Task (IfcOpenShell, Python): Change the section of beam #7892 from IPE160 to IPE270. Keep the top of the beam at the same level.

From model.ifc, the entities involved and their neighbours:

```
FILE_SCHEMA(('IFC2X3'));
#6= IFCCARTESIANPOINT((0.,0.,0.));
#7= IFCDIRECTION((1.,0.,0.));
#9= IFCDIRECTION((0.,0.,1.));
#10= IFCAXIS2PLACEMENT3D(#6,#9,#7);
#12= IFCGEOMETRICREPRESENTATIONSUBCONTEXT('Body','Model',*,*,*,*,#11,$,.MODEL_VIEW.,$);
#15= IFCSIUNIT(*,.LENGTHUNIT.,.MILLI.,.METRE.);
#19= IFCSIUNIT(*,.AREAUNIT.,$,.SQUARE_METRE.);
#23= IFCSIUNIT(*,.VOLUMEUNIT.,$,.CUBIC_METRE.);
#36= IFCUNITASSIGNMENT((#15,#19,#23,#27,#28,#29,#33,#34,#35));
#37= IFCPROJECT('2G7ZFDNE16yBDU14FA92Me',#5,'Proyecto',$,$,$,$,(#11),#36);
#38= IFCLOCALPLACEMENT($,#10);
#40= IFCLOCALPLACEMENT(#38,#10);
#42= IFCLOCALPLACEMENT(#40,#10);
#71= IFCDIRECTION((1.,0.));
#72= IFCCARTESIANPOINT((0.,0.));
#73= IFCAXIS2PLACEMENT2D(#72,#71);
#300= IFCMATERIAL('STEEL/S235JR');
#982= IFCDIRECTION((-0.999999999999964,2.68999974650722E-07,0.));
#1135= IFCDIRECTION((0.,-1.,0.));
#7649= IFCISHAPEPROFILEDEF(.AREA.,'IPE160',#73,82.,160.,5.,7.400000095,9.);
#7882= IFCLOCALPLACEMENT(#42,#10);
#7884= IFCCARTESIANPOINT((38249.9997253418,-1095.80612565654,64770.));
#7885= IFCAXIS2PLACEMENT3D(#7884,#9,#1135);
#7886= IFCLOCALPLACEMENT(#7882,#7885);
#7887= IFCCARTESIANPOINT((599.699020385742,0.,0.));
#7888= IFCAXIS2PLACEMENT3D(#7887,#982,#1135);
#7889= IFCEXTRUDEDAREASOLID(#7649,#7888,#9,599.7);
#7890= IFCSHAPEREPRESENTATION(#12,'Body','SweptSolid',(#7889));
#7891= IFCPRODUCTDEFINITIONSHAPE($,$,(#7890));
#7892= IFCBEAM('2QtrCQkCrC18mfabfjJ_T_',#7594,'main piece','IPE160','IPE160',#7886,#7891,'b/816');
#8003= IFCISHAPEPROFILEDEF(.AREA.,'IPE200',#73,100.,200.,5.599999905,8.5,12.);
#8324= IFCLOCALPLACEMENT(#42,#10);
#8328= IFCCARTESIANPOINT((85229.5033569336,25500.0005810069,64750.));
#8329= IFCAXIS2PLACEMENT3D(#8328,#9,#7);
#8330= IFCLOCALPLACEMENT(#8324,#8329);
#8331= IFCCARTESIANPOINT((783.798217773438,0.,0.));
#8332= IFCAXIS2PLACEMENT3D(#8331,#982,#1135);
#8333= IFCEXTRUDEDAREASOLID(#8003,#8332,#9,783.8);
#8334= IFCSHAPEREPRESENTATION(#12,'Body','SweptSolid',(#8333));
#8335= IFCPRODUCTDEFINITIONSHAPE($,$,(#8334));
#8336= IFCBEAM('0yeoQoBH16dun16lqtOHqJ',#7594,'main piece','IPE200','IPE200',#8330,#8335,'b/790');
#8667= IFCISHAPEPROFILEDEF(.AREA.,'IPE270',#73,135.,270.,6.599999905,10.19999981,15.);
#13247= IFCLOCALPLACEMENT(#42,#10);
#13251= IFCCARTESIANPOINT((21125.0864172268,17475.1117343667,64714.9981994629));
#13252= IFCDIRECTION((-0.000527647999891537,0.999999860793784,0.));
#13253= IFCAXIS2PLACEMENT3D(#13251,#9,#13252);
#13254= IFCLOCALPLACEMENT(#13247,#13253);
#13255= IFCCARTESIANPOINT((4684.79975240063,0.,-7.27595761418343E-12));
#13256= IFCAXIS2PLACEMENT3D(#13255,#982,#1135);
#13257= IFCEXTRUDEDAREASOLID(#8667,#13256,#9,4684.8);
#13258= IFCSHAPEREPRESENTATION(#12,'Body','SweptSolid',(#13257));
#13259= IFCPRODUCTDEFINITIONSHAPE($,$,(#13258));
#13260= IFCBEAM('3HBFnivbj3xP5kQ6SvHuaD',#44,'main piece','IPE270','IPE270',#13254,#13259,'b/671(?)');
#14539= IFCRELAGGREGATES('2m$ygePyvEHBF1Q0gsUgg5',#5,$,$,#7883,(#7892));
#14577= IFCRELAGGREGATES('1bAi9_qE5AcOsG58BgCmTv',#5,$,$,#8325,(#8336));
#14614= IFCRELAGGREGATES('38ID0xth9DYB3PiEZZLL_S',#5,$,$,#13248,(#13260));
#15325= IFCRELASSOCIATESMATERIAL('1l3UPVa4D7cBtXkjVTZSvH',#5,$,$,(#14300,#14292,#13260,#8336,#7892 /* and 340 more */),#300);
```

```python
import ifcopenshell
import ifcopenshell.util.element
import ifcopenshell.util.representation

model = ifcopenshell.open("model.ifc")

member = model.by_guid("2QtrCQkCrC18mfabfjJ_T_")
source = next(p for p in model.by_type("IfcIShapeProfileDef") if p.ProfileName == "IPE270")

body = ifcopenshell.util.representation.get_representation(member, "Model", "Body")
solid = body.Items[0]
old_profile = solid.SweptArea

# Copy the section's sizes but keep this member's own profile position.
profile = ifcopenshell.util.element.copy(model, source)
# Profiles are centred, so shift by half the change in depth to hold the top.
shift = (old_profile.OverallDepth - profile.OverallDepth) / 2
x, y = old_profile.Position.Location.Coordinates
up = (0.0, 1.0)  # upwards, in the solid's own plane
location = model.createIfcCartesianPoint((x + up[0] * shift, y + up[1] * shift))
profile.Position = model.createIfcAxis2Placement2D(location, old_profile.Position.RefDirection)
solid.SweptArea = profile
if not model.get_total_inverses(old_profile):
    ifcopenshell.util.element.remove_deep2(model, old_profile)
member.Description = member.Description.replace("IPE160", "IPE270")
member.ObjectType = member.ObjectType.replace("IPE160", "IPE270")

print(solid.SweptArea)

model.write("model_rev.ifc")
```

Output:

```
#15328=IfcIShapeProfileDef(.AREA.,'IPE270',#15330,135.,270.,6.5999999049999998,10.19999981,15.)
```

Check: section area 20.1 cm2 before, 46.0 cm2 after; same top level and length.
